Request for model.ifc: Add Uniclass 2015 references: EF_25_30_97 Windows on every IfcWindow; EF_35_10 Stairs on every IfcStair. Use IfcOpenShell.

First a look at what the model holds.

```python
import ifcopenshell

model = ifcopenshell.open("model.ifc")
print(model.schema)
print("classifications:", [c.Name for c in model.by_type("IfcClassification")])
for ifc_class in ("IfcDoor", "IfcRoof", "IfcStair", "IfcWall", "IfcWindow"):
    print(ifc_class, len(model.by_type(ifc_class)))
```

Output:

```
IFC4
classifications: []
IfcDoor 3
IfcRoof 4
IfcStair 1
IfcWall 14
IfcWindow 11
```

```python
import ifcopenshell
import ifcopenshell.api.classification

model = ifcopenshell.open("model.ifc")

system = ifcopenshell.api.classification.add_classification(model, classification="Uniclass 2015")

codes = {
    "IfcWindow": ("EF_25_30_97", "Windows"),
    "IfcStair": ("EF_35_10", "Stairs"),
}
for ifc_class, (code, name) in codes.items():
    products = model.by_type(ifc_class)
    ifcopenshell.api.classification.add_reference(
        model, products=products, classification=system, identification=code, name=name
    )
    print(code, len(products))

model.write("model_v2.ifc")
```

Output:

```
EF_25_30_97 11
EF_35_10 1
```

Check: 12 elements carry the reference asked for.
